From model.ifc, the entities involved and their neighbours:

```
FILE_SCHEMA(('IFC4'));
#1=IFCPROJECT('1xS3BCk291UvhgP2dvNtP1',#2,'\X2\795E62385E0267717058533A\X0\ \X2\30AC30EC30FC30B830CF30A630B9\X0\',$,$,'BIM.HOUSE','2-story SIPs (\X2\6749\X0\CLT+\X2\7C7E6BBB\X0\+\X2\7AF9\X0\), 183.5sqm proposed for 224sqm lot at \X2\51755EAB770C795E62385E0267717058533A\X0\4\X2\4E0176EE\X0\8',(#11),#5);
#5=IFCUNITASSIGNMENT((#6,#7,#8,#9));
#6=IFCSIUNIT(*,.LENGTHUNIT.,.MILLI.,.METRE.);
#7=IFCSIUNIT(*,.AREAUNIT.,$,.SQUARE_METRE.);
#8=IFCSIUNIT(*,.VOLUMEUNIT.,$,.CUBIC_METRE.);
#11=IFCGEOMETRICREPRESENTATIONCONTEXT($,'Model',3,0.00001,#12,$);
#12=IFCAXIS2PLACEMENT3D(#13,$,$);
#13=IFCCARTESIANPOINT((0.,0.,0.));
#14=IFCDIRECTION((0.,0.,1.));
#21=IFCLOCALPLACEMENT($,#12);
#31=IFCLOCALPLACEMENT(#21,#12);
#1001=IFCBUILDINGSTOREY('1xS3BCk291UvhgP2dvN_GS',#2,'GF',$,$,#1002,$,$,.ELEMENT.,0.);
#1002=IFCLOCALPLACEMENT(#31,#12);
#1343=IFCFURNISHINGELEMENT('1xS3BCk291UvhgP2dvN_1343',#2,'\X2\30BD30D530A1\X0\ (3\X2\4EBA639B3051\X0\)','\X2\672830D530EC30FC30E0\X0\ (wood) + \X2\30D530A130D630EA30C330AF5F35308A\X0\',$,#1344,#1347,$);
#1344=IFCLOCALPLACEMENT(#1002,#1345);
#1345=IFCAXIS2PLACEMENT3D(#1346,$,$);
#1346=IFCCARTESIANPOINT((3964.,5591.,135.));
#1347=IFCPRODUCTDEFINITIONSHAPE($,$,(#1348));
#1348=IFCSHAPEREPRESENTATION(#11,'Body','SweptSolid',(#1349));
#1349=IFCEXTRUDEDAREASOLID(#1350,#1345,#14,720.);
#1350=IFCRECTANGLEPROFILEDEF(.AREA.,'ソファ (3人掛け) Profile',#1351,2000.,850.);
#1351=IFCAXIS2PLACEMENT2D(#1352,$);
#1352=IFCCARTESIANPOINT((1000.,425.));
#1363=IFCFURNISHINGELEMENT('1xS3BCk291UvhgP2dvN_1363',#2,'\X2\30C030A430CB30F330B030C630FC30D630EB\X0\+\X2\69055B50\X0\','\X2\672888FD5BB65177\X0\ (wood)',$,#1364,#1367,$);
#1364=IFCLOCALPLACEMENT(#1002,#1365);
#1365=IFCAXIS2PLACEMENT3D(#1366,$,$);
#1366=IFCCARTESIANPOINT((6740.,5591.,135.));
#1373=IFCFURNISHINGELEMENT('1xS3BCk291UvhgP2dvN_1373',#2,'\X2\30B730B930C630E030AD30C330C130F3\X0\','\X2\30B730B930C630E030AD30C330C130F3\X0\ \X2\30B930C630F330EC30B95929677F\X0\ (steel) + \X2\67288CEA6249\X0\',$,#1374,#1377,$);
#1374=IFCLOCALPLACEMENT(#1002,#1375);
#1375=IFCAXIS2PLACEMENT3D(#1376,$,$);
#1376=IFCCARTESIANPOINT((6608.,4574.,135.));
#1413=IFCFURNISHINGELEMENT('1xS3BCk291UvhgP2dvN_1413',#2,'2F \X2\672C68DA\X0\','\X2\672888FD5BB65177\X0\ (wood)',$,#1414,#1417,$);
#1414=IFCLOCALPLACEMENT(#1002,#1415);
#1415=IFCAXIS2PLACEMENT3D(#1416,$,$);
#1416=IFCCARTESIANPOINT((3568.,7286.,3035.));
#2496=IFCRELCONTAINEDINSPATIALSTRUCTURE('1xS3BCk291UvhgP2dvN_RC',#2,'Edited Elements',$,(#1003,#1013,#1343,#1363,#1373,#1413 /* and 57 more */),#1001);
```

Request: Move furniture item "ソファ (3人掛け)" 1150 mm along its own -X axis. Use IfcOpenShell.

```python
import ifcopenshell
import ifcopenshell.api.geometry
import ifcopenshell.util.placement

model = ifcopenshell.open("model.ifc")

item = model.by_guid("1xS3BCk291UvhgP2dvN_1343")
matrix = ifcopenshell.util.placement.get_local_placement(item.ObjectPlacement)
matrix[:3, 3] -= matrix[:3, 0] * 1150.0
ifcopenshell.api.geometry.edit_object_placement(model, product=item, matrix=matrix, is_si=False)

print(ifcopenshell.util.placement.get_local_placement(item.ObjectPlacement).round(3) + 0.0)

model.write("model_edited.ifc")
```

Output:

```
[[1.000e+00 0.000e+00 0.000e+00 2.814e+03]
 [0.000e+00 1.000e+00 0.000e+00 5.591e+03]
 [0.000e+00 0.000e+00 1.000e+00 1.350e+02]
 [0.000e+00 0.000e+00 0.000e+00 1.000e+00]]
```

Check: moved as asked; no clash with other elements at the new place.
